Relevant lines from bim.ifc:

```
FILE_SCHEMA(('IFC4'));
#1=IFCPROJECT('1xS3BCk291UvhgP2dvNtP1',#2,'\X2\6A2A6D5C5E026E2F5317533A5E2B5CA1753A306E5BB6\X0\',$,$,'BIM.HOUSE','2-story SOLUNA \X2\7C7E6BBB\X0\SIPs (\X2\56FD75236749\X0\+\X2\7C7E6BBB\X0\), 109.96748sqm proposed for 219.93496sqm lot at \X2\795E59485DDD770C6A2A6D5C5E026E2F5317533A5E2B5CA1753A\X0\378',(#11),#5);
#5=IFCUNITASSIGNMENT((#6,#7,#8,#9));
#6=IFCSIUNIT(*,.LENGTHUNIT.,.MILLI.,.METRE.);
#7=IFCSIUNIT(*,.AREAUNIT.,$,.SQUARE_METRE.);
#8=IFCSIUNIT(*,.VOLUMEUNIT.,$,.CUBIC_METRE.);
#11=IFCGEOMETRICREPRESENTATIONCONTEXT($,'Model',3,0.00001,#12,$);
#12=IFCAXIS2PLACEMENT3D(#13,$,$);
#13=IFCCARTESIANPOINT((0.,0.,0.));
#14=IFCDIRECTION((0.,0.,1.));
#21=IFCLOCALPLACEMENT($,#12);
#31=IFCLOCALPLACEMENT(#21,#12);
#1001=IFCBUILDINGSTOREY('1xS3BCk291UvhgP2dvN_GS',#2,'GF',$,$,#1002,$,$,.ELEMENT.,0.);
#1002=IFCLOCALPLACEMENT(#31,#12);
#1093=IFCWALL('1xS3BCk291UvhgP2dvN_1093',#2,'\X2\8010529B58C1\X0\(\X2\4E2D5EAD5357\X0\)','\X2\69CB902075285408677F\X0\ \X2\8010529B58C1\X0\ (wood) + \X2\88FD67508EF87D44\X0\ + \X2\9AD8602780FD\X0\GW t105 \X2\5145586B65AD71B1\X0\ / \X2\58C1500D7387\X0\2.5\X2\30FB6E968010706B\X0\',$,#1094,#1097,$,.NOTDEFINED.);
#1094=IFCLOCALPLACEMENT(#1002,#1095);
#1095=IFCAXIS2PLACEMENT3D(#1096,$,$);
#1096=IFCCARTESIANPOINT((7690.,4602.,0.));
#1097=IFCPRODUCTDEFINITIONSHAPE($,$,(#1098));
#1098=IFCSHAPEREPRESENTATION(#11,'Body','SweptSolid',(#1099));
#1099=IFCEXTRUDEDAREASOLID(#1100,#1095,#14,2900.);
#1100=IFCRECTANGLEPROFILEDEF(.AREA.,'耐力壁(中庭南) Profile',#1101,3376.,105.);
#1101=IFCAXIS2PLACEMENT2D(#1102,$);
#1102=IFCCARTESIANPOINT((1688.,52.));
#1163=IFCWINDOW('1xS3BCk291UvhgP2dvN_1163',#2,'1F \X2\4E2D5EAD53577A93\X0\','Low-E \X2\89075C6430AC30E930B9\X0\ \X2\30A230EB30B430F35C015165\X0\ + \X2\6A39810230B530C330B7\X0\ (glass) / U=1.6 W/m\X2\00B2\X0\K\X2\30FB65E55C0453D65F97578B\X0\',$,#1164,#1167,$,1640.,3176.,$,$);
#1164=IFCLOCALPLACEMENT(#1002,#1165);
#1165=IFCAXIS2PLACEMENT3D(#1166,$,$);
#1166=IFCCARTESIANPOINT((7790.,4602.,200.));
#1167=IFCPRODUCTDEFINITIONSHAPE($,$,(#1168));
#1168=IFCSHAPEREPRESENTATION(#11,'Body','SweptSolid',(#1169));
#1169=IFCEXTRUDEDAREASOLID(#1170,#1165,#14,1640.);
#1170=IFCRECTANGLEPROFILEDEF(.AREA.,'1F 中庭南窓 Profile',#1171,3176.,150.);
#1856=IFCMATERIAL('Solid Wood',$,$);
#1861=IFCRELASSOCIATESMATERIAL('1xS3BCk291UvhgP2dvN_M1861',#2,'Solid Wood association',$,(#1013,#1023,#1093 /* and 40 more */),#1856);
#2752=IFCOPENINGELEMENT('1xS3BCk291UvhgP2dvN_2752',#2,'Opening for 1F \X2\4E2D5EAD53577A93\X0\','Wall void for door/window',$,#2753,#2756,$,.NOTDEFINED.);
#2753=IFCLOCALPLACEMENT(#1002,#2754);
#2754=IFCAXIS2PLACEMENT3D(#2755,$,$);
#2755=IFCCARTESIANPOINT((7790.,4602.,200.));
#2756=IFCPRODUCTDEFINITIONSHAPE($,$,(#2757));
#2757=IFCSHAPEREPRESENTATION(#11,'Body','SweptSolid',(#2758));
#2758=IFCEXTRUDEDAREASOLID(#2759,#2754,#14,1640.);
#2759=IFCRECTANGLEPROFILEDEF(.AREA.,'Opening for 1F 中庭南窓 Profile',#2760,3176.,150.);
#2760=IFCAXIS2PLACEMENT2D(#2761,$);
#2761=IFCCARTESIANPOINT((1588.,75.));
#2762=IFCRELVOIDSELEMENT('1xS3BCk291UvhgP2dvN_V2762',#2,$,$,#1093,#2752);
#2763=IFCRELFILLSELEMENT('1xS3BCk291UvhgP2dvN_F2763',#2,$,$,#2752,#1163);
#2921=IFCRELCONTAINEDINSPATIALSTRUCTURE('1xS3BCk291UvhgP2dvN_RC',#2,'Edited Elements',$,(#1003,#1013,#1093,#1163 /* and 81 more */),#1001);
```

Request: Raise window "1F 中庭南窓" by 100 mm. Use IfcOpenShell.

```python
import numpy as np
import ifcopenshell
import ifcopenshell.api.geometry
import ifcopenshell.util.placement
import ifcopenshell.util.unit

model = ifcopenshell.open("bim.ifc")
unit_scale = ifcopenshell.util.unit.calculate_unit_scale(model)

window = model.by_guid("1xS3BCk291UvhgP2dvN_1163")
opening = window.FillsVoids[0].RelatingOpeningElement
dz = 100.0

shift = np.array([0.0, 0.0, dz])
# The window is not placed relative to its opening, so move both.
for product in (opening, window):
    matrix = ifcopenshell.util.placement.get_local_placement(product.ObjectPlacement)
    matrix[:3, 3] += shift
    ifcopenshell.api.geometry.edit_object_placement(model, product=product, matrix=matrix, is_si=False)

print(f"moved by {dz * unit_scale:+.3f} m")

model.write("bim-out.ifc")
```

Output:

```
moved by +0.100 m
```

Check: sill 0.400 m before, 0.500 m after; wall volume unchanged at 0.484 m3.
